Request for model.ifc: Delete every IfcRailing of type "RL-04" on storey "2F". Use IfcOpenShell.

First a look at what the model holds.

```python
import ifcopenshell
import ifcopenshell.util.element

model = ifcopenshell.open("model.ifc")
print(model.schema)
storey = next(s for s in model.by_type("IfcBuildingStorey") if s.Name == "2F")
railings = [e for e in ifcopenshell.util.element.get_decomposition(storey) if e.is_a("IfcRailing")]
seen = {}
for e in railings:
    element_type = ifcopenshell.util.element.get_type(e)
    name = element_type.Name if element_type not in (None, e) else None
    seen[name] = seen.get(name, 0) + 1
for name, count in sorted(seen.items(), key=str):
    print(count, "x", name)
```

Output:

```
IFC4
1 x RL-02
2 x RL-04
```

```python
import ifcopenshell
import ifcopenshell.api.root
import ifcopenshell.util.element

model = ifcopenshell.open("model.ifc")

storey = next(s for s in model.by_type("IfcBuildingStorey") if s.Name == "2F")
railings = [e for e in ifcopenshell.util.element.get_decomposition(storey) if e.is_a("IfcRailing")]
targets = [e for e in railings if (t := ifcopenshell.util.element.get_type(e)) not in (None, e) and t.Name == "RL-04"]

for e in targets:
    ifcopenshell.api.root.remove_product(model, product=e)
print(len(targets), "removed")

model.write("model_updated.ifc")
```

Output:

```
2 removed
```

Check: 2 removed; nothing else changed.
